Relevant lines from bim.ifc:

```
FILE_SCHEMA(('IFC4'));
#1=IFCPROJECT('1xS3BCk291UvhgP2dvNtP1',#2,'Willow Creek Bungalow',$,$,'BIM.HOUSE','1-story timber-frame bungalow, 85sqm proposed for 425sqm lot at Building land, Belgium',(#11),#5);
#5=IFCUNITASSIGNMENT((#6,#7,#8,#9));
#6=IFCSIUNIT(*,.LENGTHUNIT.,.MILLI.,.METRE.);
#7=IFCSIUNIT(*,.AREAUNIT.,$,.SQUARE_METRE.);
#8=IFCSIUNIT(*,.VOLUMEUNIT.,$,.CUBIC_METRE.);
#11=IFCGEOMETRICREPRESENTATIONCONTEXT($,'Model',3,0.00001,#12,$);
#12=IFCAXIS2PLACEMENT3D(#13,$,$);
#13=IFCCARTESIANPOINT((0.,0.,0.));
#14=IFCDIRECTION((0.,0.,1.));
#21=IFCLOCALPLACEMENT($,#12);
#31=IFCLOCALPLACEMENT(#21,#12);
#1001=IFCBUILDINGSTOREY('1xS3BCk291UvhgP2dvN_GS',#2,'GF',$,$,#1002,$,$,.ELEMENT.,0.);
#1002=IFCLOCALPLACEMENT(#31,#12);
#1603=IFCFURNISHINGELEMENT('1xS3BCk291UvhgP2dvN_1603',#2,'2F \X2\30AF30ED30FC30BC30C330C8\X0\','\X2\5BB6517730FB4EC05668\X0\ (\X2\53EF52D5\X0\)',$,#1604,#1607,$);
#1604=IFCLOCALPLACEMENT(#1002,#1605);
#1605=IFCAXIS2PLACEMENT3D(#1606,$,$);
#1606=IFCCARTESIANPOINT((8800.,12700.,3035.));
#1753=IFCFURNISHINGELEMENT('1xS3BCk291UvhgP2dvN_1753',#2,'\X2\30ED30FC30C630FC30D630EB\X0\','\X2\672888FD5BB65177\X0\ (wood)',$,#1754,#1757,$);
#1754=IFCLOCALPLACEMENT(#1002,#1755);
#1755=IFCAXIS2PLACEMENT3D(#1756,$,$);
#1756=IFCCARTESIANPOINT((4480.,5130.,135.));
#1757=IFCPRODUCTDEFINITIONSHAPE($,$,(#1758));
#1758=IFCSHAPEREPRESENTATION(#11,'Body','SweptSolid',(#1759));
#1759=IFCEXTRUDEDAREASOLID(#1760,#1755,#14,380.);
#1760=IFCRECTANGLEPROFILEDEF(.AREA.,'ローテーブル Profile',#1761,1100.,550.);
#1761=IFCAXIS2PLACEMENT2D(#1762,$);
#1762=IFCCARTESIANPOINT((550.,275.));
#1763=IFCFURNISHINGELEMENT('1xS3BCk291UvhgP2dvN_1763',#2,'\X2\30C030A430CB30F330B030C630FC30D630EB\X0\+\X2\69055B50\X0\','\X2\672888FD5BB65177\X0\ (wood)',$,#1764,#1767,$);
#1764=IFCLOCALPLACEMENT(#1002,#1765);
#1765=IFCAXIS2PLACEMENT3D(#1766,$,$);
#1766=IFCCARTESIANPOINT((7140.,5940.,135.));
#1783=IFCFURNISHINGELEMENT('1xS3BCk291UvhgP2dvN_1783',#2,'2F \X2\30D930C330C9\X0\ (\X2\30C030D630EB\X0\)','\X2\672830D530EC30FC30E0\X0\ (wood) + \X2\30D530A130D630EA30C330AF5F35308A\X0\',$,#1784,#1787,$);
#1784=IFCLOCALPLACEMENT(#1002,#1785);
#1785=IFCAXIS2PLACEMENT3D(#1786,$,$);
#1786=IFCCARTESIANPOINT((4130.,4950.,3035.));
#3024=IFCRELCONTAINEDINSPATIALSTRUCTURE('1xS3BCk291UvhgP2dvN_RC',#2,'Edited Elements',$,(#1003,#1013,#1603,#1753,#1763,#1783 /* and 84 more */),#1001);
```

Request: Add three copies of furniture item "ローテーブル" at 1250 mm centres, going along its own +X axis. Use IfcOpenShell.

```python
import ifcopenshell
import ifcopenshell.api.geometry
import ifcopenshell.api.root
import ifcopenshell.util.element
import ifcopenshell.util.placement

model = ifcopenshell.open("bim.ifc")


def reuse_history(source, copy):
    """copy_class also copies each property set's owner history, people and application; keep the originals."""
    for rel in copy.IsDefinedBy:
        if rel.is_a("IfcRelDefinesByProperties") and (history := rel.RelatingPropertyDefinition.OwnerHistory):
            rel.RelatingPropertyDefinition.OwnerHistory = source.OwnerHistory
            ifcopenshell.util.element.remove_deep2(model, history)


source = model.by_guid("1xS3BCk291UvhgP2dvN_1753")
base = ifcopenshell.util.placement.get_local_placement(source.ObjectPlacement)
step = base[:3, 0] * 1250.0

for i in range(1, 4):
    copy = ifcopenshell.api.root.copy_class(model, product=source)
    copy.Representation = ifcopenshell.util.element.copy_deep(
        model, source.Representation, exclude=["IfcGeometricRepresentationContext", "IfcRepresentationMap"]
    )
    reuse_history(source, copy)
    matrix = base.copy()
    matrix[:3, 3] += i * step
    print("added at", matrix[:3, 3].round(3) + 0.0)
    ifcopenshell.api.geometry.edit_object_placement(model, product=copy, matrix=matrix, is_si=False)

model.write("bim_rev.ifc")
```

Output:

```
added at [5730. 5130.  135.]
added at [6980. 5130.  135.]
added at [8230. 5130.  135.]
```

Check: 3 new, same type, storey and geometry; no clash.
